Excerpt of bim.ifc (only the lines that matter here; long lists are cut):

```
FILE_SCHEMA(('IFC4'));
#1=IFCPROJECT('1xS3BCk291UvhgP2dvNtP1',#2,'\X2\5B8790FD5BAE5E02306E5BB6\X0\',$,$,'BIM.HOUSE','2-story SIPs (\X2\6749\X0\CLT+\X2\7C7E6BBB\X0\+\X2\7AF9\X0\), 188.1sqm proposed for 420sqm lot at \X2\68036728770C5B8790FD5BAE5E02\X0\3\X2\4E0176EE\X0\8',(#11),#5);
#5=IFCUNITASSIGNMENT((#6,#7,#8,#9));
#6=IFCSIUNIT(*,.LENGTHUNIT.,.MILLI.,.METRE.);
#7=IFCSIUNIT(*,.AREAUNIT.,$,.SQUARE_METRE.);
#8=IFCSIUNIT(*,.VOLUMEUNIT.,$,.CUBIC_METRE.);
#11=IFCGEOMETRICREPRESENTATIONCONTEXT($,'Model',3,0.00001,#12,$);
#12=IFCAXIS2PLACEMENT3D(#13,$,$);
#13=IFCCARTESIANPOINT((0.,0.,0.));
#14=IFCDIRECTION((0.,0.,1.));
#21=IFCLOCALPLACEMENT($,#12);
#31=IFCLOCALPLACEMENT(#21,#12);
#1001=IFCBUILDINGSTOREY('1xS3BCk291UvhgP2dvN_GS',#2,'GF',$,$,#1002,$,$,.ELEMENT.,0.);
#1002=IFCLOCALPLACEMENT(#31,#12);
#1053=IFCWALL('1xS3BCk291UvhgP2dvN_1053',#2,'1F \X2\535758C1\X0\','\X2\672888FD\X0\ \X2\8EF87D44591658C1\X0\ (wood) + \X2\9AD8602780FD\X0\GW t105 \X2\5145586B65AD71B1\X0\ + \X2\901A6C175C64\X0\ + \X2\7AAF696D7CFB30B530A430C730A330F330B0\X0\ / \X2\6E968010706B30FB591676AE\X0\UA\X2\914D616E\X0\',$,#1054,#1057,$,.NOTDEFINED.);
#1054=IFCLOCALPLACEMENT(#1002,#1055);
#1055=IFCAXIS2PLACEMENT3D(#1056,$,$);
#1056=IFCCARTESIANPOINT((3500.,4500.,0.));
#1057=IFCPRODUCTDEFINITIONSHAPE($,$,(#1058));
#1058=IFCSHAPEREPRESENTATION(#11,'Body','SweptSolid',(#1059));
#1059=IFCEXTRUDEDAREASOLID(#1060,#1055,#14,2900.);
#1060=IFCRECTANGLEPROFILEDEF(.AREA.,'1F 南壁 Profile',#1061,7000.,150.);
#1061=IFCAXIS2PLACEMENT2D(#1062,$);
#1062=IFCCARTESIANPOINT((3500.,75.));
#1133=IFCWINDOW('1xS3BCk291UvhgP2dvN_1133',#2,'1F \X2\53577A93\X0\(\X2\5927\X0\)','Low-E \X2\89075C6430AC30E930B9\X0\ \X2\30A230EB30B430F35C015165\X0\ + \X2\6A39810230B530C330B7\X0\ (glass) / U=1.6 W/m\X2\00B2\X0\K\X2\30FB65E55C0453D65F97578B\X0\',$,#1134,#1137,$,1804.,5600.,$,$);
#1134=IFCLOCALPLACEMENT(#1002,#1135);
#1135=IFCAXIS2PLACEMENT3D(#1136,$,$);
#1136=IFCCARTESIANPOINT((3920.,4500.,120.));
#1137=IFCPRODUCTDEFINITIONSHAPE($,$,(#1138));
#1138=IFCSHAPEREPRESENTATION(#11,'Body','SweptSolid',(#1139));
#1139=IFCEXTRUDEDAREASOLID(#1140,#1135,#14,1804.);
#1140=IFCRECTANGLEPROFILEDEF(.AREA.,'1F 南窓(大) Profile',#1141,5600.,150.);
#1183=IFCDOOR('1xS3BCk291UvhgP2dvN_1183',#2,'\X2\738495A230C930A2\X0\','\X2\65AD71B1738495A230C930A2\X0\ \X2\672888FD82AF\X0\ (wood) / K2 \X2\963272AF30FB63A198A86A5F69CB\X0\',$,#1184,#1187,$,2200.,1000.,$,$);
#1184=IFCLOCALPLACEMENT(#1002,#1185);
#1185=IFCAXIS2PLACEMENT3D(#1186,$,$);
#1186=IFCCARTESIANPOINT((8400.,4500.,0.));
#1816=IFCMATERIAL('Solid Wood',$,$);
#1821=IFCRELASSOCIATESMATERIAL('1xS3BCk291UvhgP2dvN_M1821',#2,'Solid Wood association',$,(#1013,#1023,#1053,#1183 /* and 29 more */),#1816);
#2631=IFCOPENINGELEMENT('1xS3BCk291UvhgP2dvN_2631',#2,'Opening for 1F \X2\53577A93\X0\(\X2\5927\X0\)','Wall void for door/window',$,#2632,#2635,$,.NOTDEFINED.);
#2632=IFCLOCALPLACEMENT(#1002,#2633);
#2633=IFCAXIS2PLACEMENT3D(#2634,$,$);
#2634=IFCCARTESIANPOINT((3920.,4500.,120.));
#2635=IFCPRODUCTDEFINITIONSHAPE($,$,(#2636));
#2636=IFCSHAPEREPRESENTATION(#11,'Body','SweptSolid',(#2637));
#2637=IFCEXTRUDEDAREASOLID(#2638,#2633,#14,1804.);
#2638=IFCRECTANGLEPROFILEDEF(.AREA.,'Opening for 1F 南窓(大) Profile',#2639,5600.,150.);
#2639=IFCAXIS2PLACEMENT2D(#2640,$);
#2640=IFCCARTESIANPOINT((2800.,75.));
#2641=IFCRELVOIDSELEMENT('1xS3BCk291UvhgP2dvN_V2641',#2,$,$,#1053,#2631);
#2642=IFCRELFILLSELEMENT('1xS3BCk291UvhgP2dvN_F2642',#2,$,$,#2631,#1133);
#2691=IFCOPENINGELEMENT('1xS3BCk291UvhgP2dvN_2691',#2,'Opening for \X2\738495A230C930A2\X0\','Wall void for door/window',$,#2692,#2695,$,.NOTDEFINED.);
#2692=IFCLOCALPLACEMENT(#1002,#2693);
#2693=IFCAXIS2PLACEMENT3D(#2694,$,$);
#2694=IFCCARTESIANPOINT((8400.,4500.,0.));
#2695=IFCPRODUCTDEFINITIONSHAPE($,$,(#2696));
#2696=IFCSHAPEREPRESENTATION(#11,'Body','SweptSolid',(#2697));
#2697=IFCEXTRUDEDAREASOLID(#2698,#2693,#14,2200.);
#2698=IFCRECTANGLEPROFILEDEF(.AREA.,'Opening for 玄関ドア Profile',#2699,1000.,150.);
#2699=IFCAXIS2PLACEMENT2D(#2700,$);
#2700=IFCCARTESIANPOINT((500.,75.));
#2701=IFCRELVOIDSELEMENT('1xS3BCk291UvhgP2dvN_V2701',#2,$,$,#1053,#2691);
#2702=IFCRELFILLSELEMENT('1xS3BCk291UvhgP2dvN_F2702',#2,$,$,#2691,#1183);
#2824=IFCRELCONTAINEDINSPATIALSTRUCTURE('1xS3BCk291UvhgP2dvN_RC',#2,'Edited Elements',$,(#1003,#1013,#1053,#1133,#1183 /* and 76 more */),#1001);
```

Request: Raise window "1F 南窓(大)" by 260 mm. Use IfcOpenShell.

```python
import numpy as np
import ifcopenshell
import ifcopenshell.api.geometry
import ifcopenshell.util.placement
import ifcopenshell.util.unit

model = ifcopenshell.open("bim.ifc")
unit_scale = ifcopenshell.util.unit.calculate_unit_scale(model)

window = model.by_guid("1xS3BCk291UvhgP2dvN_1133")
opening = window.FillsVoids[0].RelatingOpeningElement
dz = 0.26 / unit_scale

shift = np.array([0.0, 0.0, dz])
# The window is not placed relative to its opening, so move both.
for product in (opening, window):
    matrix = ifcopenshell.util.placement.get_local_placement(product.ObjectPlacement)
    matrix[:3, 3] += shift
    ifcopenshell.api.geometry.edit_object_placement(model, product=product, matrix=matrix, is_si=False)

print(f"moved by {dz * unit_scale:+.3f} m")

model.write("bim_v2.ifc")
```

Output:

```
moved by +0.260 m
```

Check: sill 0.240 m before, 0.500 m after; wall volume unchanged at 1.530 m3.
